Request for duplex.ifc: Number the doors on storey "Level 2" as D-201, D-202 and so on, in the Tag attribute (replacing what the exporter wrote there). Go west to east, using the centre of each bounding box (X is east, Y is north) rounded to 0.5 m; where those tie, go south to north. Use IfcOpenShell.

First a look at what the model holds.

```python
import ifcopenshell
import ifcopenshell.util.element
import ifcopenshell.util.placement

model = ifcopenshell.open("duplex.ifc")
print(model.schema)
storey = next(s for s in model.by_type("IfcBuildingStorey") if s.Name == "Level 2")
doors = [e for e in ifcopenshell.util.element.get_decomposition(storey) if e.is_a("IfcDoor")]
for e in sorted(doors, key=lambda e: e.id()):
    origin = ifcopenshell.util.placement.get_local_placement(e.ObjectPlacement)[:3, 3]
    print(e.id(), e.Tag, e.Name, origin.round(2) + 0.0, sep=" | ")
```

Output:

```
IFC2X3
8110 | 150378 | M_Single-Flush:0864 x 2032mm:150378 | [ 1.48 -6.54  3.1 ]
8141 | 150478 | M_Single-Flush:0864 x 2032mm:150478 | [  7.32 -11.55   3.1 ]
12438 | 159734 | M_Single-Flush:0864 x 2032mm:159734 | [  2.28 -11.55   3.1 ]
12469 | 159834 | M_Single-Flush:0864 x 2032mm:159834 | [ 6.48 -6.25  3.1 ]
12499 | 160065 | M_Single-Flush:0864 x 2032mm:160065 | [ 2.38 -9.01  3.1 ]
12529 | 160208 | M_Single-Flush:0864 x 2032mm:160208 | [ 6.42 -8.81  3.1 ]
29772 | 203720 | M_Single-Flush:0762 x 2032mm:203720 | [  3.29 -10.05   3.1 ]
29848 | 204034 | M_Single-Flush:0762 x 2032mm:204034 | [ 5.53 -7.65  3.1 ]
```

```python
import ifcopenshell
import ifcopenshell.geom
import ifcopenshell.util.element
import ifcopenshell.util.shape

model = ifcopenshell.open("duplex.ifc")
settings = ifcopenshell.geom.settings()
settings.set("use-world-coords", True)


def centre(element):
    shape = ifcopenshell.geom.create_shape(settings, element)
    return ifcopenshell.util.shape.get_bbox_centroid(shape.geometry)


storey = next(s for s in model.by_type("IfcBuildingStorey") if s.Name == "Level 2")
doors = [e for e in ifcopenshell.util.element.get_decomposition(storey) if e.is_a("IfcDoor")]

# Insertion points can sit at a corner or the storey origin, so sort by the geometry (in metres).
centres = {e: centre(e) for e in doors}
doors.sort(key=lambda e: (round(centres[e][0] / 0.5), centres[e][1]))

for i, e in enumerate(doors, start=1):
    number = f"D-2{i:02d}"
    e.Tag = number
    print(e.id(), number)

model.write("duplex-out.ifc")
```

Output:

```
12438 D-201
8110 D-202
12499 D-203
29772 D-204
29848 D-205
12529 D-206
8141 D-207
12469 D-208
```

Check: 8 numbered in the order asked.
